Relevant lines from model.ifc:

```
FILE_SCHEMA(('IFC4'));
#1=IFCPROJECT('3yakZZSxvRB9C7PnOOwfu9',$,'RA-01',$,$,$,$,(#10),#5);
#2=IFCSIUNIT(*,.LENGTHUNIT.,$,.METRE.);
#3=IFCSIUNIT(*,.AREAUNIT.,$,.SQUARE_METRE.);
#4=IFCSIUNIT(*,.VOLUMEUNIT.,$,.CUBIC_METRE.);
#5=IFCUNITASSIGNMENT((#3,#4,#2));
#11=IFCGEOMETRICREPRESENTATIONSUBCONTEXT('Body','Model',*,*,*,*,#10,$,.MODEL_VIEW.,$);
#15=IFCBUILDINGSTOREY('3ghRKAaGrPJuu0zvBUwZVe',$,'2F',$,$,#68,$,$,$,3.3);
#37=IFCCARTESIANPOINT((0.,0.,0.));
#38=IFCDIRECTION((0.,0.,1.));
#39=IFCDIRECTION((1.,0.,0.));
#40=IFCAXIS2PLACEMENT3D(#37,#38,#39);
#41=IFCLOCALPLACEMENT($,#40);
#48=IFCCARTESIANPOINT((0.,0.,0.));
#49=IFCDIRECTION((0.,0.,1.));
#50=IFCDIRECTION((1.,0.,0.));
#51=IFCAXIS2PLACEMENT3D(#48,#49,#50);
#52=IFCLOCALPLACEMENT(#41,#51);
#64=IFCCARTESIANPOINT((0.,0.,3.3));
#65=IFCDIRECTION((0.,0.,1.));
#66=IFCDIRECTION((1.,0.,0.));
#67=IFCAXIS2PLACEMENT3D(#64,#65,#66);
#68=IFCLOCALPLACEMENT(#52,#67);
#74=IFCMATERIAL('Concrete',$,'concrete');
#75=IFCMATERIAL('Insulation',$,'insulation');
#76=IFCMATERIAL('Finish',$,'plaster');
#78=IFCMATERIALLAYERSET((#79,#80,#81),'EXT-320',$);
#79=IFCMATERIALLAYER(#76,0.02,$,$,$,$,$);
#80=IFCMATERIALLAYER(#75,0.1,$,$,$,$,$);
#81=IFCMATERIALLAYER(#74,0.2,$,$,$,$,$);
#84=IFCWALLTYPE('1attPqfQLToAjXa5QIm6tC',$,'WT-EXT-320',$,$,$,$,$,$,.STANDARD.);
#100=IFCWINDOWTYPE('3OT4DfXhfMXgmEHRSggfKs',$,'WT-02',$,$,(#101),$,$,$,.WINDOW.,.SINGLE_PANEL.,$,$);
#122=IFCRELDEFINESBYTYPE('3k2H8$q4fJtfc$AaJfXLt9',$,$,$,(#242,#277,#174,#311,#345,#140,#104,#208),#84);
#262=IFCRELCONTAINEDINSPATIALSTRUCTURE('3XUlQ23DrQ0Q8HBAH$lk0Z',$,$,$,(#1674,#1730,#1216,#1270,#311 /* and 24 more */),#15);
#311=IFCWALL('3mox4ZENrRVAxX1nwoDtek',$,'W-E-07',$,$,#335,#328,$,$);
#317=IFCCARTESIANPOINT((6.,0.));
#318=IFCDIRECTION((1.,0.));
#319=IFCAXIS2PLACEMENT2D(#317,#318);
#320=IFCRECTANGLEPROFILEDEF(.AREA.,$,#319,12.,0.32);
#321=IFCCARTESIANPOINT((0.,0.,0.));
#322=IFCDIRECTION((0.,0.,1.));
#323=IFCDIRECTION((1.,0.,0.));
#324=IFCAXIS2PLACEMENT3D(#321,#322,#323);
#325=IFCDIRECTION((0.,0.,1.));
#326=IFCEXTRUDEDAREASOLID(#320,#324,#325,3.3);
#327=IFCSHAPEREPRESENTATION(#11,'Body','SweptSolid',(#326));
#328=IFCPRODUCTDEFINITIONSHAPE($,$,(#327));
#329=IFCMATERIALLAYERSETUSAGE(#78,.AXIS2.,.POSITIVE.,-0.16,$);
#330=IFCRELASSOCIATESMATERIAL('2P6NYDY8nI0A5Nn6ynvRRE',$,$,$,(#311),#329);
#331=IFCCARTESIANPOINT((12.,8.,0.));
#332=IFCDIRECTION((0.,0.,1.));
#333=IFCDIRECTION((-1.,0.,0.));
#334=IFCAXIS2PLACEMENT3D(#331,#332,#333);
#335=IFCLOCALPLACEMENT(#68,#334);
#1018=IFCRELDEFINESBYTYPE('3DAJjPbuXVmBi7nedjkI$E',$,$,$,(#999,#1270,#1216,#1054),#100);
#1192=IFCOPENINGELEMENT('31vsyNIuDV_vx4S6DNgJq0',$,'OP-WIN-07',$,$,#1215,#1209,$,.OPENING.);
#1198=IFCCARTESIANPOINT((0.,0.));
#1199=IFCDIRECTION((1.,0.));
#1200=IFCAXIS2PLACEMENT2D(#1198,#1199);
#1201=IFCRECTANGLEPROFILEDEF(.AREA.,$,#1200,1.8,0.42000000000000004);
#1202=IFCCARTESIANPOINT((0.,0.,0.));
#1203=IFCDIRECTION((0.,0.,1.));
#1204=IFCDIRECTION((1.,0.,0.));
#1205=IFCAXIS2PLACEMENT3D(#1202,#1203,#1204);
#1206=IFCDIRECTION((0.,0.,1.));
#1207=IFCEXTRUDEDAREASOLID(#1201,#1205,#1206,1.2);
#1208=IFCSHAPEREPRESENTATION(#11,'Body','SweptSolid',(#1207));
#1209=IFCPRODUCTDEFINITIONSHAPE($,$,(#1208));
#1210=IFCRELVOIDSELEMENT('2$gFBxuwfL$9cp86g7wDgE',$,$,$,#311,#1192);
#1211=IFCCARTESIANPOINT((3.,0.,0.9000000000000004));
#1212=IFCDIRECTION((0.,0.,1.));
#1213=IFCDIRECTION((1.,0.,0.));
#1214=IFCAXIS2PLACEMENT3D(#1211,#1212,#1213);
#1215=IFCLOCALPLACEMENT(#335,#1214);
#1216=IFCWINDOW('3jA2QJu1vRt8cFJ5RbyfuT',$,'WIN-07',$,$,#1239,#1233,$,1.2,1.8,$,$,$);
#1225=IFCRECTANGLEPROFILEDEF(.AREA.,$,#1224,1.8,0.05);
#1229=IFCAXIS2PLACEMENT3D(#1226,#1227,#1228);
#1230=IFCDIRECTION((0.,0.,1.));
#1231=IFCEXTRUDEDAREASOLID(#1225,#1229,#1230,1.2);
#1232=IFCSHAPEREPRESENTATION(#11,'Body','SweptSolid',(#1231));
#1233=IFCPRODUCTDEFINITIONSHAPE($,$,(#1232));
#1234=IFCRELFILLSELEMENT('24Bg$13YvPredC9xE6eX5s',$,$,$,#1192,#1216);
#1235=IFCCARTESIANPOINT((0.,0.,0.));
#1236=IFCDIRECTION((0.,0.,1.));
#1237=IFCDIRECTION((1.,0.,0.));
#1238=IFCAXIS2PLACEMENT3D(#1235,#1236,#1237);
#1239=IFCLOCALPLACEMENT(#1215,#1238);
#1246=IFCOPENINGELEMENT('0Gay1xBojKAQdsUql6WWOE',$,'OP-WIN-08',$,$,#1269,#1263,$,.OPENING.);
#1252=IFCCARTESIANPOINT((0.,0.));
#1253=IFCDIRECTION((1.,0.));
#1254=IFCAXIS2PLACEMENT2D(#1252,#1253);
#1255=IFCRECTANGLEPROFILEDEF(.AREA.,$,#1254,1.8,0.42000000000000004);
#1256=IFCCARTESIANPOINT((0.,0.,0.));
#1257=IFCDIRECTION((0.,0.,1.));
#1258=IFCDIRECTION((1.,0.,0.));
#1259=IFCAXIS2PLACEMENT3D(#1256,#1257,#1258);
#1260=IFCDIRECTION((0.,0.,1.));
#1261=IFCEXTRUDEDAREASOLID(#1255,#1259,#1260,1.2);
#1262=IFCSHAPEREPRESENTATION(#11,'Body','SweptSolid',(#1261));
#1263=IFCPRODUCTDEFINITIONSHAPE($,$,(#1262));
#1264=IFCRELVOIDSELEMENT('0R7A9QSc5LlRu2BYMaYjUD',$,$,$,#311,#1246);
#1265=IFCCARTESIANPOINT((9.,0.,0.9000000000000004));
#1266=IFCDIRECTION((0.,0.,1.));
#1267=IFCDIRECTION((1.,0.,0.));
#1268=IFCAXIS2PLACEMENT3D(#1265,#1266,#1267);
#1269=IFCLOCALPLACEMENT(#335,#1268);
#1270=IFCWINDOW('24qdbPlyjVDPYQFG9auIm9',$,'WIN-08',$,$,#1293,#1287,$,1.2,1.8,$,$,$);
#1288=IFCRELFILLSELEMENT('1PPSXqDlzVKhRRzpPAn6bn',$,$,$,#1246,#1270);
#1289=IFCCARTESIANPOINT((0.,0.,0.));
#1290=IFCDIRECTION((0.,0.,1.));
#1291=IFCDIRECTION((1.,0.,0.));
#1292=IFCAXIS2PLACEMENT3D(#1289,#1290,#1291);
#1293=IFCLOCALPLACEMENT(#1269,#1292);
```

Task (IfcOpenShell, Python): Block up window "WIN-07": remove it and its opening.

```python
import ifcopenshell
import ifcopenshell.api.feature
import ifcopenshell.api.root
import ifcopenshell.geom
import ifcopenshell.util.shape

model = ifcopenshell.open("model.ifc")
settings = ifcopenshell.geom.settings()


def volume(element):
    """Net volume in cubic metres, openings subtracted."""
    shape = ifcopenshell.geom.create_shape(settings, element)
    return ifcopenshell.util.shape.get_volume(shape.geometry)


window = model.by_guid("3jA2QJu1vRt8cFJ5RbyfuT")
opening = window.FillsVoids[0].RelatingOpeningElement
wall = opening.VoidsElements[0].RelatingBuildingElement
before = volume(wall)

ifcopenshell.api.root.remove_product(model, product=window)
ifcopenshell.api.feature.remove_feature(model, feature=opening)

after = volume(wall)

print(f"wall volume {before:.3f} -> {after:.3f} m3")

model.write("model_updated.ifc")
```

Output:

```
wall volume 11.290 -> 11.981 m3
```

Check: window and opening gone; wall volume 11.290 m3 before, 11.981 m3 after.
